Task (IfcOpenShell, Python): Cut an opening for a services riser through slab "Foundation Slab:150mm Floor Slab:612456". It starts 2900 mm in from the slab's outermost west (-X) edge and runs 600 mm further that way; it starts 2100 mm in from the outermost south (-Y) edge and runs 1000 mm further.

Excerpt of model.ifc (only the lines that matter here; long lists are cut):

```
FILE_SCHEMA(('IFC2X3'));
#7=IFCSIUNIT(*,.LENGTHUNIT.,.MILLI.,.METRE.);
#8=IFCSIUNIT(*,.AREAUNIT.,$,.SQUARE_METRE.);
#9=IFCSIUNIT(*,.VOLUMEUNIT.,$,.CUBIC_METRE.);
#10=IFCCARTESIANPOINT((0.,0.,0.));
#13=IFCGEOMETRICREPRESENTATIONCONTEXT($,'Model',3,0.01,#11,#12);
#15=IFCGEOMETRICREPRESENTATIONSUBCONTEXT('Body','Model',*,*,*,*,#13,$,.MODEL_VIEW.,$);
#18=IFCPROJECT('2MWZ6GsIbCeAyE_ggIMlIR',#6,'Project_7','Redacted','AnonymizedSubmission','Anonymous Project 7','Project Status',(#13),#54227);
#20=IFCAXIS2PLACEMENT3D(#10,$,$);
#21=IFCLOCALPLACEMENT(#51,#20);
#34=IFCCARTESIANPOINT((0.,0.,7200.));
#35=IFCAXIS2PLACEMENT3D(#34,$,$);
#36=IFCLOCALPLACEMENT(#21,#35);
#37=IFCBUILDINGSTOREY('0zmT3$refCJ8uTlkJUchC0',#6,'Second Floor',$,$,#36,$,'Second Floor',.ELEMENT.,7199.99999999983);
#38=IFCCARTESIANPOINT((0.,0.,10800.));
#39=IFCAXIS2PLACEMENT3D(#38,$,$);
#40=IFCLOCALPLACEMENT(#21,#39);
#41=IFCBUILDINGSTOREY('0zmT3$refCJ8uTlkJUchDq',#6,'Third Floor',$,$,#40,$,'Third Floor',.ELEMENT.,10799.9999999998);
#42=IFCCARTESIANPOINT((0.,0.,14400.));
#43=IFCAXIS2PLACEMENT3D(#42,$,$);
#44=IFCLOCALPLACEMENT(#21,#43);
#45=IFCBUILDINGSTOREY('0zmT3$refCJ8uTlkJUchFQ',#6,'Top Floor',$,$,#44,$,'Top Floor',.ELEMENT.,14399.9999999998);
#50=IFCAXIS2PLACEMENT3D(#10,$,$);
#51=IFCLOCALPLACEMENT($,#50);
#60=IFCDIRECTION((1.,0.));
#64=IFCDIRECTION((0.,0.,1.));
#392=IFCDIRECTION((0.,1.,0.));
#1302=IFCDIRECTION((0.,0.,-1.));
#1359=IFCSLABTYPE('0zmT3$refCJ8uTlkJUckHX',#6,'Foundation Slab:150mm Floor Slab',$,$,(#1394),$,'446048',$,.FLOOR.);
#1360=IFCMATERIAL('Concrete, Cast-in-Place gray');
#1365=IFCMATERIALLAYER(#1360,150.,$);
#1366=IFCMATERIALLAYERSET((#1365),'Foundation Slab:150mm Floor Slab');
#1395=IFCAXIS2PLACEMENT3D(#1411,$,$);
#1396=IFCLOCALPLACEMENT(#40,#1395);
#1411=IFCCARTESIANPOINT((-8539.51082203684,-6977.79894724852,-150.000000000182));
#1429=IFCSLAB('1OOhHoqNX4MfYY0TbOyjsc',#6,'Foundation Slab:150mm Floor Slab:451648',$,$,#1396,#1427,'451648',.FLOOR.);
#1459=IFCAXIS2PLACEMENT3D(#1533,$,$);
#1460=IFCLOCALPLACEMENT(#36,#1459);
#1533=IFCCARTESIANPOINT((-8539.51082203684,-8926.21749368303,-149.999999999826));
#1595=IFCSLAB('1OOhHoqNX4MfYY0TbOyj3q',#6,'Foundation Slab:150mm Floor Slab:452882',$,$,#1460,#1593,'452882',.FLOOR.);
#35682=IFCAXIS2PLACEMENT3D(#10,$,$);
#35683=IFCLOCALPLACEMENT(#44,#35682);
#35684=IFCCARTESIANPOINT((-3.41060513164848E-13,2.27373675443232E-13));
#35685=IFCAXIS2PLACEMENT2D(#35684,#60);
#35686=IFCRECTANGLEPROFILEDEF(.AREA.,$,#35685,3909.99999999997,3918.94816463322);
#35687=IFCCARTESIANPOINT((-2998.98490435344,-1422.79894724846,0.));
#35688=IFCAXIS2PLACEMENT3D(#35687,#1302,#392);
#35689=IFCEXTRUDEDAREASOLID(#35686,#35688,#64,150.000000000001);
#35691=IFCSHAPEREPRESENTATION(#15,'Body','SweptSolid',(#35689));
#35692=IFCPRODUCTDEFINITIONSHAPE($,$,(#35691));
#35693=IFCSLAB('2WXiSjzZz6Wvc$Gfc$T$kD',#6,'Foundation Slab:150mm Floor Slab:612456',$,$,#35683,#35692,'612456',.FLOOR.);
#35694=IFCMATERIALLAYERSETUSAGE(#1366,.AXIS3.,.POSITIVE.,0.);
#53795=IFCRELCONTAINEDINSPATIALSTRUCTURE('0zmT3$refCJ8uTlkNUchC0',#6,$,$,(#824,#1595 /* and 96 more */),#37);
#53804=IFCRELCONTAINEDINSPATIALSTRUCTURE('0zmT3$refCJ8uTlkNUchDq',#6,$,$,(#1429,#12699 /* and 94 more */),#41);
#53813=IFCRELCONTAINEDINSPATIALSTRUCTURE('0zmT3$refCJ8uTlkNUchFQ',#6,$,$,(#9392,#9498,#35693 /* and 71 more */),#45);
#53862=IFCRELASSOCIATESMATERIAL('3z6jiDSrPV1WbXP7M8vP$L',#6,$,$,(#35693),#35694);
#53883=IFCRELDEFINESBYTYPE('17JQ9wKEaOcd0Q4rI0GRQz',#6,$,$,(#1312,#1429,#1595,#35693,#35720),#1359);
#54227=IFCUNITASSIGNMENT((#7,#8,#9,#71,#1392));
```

```python
import numpy as np
import ifcopenshell
import ifcopenshell.api.feature
import ifcopenshell.api.geometry
import ifcopenshell.api.root
import ifcopenshell.geom
import ifcopenshell.util.placement
import ifcopenshell.util.representation
import ifcopenshell.util.shape
import ifcopenshell.util.unit

model = ifcopenshell.open("model.ifc")
unit_scale = ifcopenshell.util.unit.calculate_unit_scale(model)
settings = ifcopenshell.geom.settings()


def volume(element):
    """Net volume in cubic metres, openings subtracted."""
    shape = ifcopenshell.geom.create_shape(settings, element)
    return ifcopenshell.util.shape.get_volume(shape.geometry)


slab = model.by_guid("2WXiSjzZz6Wvc$Gfc$T$kD")
before = volume(slab)

# Extent in the slab's own axes, in metres. The edges named are its -X and -Y sides.
slab_shape = ifcopenshell.geom.create_shape(settings, slab)
vertices = ifcopenshell.util.shape.get_vertices(slab_shape.geometry)
x_min, y_min, bottom = vertices.min(axis=0)
top = vertices[:, 2].max()

opening = ifcopenshell.api.root.create_entity(model, ifc_class="IfcOpeningElement", name="Services riser opening")
context = ifcopenshell.util.representation.get_context(model, "Model", "Body", "MODEL_VIEW")
width, depth = 0.6, 1
outline = [(0.0, 0.0), (width, 0.0), (width, depth), (0.0, depth), (0.0, 0.0)]
# Overshoot both faces by 50 mm so the cut is clean.
shape = ifcopenshell.api.geometry.add_slab_representation(
    model, context=context, depth=top - bottom + 0.1, polyline=outline
)
ifcopenshell.api.geometry.assign_representation(model, product=opening, representation=shape)

matrix = ifcopenshell.util.placement.get_local_placement(slab.ObjectPlacement)
matrix[:, 3] = matrix @ np.append(np.array([x_min + 2.9, y_min + 2.1, bottom - 0.05]) / unit_scale, 1.0)
ifcopenshell.api.geometry.edit_object_placement(model, product=opening, matrix=matrix, is_si=False)
ifcopenshell.api.feature.add_feature(model, feature=opening, element=slab)

after = volume(slab)

print(f"slab volume {before:.3f} -> {after:.3f} m3")

model.write("model_edited.ifc")
```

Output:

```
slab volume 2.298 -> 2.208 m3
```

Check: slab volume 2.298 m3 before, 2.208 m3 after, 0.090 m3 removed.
